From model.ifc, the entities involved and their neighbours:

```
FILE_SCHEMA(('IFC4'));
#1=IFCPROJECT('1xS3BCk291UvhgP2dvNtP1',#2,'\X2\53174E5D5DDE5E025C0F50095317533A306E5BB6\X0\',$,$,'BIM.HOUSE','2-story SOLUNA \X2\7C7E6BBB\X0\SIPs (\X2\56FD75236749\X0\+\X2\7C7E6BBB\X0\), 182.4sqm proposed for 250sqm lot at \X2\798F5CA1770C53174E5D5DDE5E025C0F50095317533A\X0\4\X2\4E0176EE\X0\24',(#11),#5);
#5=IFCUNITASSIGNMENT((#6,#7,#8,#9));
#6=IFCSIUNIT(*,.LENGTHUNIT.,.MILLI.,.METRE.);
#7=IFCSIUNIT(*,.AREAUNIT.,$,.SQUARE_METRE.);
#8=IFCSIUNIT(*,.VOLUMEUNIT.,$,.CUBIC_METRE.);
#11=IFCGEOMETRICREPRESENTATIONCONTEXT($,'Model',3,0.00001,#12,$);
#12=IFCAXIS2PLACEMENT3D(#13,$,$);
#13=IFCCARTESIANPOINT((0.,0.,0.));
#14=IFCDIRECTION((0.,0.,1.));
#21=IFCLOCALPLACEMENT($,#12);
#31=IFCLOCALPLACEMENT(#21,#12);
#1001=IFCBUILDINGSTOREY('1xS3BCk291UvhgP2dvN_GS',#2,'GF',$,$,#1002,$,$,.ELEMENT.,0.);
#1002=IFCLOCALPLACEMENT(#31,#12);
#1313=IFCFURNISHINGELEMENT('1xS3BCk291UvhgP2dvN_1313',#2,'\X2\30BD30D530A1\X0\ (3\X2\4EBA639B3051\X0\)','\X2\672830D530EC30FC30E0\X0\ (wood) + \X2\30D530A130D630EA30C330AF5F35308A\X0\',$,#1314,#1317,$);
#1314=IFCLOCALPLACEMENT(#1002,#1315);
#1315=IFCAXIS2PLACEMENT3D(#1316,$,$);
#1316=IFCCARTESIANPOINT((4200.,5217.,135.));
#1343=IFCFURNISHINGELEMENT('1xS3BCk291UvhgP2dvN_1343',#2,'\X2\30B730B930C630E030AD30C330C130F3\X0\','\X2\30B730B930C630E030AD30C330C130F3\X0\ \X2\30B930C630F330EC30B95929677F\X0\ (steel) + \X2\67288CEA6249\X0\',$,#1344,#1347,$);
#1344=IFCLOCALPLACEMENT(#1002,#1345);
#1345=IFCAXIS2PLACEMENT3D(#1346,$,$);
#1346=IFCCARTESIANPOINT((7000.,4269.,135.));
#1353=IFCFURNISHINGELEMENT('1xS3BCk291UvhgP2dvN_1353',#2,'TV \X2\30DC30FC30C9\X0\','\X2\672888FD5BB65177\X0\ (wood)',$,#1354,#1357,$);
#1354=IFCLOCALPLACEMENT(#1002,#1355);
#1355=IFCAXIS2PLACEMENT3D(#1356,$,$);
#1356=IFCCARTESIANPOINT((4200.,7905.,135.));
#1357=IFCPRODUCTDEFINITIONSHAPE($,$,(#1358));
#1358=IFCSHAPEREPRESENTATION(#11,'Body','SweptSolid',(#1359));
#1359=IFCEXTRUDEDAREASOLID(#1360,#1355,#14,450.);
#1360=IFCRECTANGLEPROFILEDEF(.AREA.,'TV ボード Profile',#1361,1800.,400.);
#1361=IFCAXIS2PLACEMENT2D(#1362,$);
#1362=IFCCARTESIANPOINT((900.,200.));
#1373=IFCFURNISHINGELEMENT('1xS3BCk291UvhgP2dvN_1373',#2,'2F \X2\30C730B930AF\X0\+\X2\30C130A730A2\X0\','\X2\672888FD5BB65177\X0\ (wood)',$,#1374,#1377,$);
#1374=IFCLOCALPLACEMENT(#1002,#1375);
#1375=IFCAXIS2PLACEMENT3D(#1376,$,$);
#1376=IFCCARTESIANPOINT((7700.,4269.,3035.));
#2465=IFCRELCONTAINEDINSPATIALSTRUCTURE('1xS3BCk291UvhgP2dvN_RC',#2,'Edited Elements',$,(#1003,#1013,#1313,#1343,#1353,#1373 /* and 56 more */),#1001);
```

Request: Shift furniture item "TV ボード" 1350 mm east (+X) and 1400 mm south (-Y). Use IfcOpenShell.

```python
import ifcopenshell
import ifcopenshell.api.geometry
import ifcopenshell.util.placement
import ifcopenshell.util.unit

model = ifcopenshell.open("model.ifc")
unit_scale = ifcopenshell.util.unit.calculate_unit_scale(model)

item = model.by_id(1353)
matrix = ifcopenshell.util.placement.get_local_placement(item.ObjectPlacement)
matrix[0, 3] += 1.35 / unit_scale
matrix[1, 3] -= 1.4 / unit_scale
ifcopenshell.api.geometry.edit_object_placement(model, product=item, matrix=matrix, is_si=False)

print(ifcopenshell.util.placement.get_local_placement(item.ObjectPlacement).round(3) + 0.0)

model.write("model_updated.ifc")
```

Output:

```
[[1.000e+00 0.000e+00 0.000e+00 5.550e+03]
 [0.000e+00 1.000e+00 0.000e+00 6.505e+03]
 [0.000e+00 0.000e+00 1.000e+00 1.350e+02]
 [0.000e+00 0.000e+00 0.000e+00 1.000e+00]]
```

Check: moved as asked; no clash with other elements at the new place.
